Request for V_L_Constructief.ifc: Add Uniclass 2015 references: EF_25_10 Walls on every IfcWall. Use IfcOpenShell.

First a look at what the model holds.

```python
import ifcopenshell

model = ifcopenshell.open("V_L_Constructief.ifc")
print(model.schema)
print("classifications:", [c.Name for c in model.by_type("IfcClassification")])
for ifc_class in ("IfcDoor", "IfcRoof", "IfcStair", "IfcWall", "IfcWindow"):
    print(ifc_class, len(model.by_type(ifc_class)))
```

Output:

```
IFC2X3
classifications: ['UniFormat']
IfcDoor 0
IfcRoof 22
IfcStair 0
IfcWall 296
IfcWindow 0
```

```python
import ifcopenshell
import ifcopenshell.api.classification

model = ifcopenshell.open("V_L_Constructief.ifc")

# IFC2X3 requires Source and Edition and has no link from the project to the system.
system = model.create_entity("IfcClassification", Source="NBS", Edition="2015", Name="Uniclass 2015")

codes = {
    "IfcWall": ("EF_25_10", "Walls"),
}
for ifc_class, (code, name) in codes.items():
    products = model.by_type(ifc_class)
    ifcopenshell.api.classification.add_reference(
        model, products=products, classification=system, identification=code, name=name
    )
    print(code, len(products))

model.write("V_L_Constructief_edited.ifc")
```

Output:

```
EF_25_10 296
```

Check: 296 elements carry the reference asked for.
